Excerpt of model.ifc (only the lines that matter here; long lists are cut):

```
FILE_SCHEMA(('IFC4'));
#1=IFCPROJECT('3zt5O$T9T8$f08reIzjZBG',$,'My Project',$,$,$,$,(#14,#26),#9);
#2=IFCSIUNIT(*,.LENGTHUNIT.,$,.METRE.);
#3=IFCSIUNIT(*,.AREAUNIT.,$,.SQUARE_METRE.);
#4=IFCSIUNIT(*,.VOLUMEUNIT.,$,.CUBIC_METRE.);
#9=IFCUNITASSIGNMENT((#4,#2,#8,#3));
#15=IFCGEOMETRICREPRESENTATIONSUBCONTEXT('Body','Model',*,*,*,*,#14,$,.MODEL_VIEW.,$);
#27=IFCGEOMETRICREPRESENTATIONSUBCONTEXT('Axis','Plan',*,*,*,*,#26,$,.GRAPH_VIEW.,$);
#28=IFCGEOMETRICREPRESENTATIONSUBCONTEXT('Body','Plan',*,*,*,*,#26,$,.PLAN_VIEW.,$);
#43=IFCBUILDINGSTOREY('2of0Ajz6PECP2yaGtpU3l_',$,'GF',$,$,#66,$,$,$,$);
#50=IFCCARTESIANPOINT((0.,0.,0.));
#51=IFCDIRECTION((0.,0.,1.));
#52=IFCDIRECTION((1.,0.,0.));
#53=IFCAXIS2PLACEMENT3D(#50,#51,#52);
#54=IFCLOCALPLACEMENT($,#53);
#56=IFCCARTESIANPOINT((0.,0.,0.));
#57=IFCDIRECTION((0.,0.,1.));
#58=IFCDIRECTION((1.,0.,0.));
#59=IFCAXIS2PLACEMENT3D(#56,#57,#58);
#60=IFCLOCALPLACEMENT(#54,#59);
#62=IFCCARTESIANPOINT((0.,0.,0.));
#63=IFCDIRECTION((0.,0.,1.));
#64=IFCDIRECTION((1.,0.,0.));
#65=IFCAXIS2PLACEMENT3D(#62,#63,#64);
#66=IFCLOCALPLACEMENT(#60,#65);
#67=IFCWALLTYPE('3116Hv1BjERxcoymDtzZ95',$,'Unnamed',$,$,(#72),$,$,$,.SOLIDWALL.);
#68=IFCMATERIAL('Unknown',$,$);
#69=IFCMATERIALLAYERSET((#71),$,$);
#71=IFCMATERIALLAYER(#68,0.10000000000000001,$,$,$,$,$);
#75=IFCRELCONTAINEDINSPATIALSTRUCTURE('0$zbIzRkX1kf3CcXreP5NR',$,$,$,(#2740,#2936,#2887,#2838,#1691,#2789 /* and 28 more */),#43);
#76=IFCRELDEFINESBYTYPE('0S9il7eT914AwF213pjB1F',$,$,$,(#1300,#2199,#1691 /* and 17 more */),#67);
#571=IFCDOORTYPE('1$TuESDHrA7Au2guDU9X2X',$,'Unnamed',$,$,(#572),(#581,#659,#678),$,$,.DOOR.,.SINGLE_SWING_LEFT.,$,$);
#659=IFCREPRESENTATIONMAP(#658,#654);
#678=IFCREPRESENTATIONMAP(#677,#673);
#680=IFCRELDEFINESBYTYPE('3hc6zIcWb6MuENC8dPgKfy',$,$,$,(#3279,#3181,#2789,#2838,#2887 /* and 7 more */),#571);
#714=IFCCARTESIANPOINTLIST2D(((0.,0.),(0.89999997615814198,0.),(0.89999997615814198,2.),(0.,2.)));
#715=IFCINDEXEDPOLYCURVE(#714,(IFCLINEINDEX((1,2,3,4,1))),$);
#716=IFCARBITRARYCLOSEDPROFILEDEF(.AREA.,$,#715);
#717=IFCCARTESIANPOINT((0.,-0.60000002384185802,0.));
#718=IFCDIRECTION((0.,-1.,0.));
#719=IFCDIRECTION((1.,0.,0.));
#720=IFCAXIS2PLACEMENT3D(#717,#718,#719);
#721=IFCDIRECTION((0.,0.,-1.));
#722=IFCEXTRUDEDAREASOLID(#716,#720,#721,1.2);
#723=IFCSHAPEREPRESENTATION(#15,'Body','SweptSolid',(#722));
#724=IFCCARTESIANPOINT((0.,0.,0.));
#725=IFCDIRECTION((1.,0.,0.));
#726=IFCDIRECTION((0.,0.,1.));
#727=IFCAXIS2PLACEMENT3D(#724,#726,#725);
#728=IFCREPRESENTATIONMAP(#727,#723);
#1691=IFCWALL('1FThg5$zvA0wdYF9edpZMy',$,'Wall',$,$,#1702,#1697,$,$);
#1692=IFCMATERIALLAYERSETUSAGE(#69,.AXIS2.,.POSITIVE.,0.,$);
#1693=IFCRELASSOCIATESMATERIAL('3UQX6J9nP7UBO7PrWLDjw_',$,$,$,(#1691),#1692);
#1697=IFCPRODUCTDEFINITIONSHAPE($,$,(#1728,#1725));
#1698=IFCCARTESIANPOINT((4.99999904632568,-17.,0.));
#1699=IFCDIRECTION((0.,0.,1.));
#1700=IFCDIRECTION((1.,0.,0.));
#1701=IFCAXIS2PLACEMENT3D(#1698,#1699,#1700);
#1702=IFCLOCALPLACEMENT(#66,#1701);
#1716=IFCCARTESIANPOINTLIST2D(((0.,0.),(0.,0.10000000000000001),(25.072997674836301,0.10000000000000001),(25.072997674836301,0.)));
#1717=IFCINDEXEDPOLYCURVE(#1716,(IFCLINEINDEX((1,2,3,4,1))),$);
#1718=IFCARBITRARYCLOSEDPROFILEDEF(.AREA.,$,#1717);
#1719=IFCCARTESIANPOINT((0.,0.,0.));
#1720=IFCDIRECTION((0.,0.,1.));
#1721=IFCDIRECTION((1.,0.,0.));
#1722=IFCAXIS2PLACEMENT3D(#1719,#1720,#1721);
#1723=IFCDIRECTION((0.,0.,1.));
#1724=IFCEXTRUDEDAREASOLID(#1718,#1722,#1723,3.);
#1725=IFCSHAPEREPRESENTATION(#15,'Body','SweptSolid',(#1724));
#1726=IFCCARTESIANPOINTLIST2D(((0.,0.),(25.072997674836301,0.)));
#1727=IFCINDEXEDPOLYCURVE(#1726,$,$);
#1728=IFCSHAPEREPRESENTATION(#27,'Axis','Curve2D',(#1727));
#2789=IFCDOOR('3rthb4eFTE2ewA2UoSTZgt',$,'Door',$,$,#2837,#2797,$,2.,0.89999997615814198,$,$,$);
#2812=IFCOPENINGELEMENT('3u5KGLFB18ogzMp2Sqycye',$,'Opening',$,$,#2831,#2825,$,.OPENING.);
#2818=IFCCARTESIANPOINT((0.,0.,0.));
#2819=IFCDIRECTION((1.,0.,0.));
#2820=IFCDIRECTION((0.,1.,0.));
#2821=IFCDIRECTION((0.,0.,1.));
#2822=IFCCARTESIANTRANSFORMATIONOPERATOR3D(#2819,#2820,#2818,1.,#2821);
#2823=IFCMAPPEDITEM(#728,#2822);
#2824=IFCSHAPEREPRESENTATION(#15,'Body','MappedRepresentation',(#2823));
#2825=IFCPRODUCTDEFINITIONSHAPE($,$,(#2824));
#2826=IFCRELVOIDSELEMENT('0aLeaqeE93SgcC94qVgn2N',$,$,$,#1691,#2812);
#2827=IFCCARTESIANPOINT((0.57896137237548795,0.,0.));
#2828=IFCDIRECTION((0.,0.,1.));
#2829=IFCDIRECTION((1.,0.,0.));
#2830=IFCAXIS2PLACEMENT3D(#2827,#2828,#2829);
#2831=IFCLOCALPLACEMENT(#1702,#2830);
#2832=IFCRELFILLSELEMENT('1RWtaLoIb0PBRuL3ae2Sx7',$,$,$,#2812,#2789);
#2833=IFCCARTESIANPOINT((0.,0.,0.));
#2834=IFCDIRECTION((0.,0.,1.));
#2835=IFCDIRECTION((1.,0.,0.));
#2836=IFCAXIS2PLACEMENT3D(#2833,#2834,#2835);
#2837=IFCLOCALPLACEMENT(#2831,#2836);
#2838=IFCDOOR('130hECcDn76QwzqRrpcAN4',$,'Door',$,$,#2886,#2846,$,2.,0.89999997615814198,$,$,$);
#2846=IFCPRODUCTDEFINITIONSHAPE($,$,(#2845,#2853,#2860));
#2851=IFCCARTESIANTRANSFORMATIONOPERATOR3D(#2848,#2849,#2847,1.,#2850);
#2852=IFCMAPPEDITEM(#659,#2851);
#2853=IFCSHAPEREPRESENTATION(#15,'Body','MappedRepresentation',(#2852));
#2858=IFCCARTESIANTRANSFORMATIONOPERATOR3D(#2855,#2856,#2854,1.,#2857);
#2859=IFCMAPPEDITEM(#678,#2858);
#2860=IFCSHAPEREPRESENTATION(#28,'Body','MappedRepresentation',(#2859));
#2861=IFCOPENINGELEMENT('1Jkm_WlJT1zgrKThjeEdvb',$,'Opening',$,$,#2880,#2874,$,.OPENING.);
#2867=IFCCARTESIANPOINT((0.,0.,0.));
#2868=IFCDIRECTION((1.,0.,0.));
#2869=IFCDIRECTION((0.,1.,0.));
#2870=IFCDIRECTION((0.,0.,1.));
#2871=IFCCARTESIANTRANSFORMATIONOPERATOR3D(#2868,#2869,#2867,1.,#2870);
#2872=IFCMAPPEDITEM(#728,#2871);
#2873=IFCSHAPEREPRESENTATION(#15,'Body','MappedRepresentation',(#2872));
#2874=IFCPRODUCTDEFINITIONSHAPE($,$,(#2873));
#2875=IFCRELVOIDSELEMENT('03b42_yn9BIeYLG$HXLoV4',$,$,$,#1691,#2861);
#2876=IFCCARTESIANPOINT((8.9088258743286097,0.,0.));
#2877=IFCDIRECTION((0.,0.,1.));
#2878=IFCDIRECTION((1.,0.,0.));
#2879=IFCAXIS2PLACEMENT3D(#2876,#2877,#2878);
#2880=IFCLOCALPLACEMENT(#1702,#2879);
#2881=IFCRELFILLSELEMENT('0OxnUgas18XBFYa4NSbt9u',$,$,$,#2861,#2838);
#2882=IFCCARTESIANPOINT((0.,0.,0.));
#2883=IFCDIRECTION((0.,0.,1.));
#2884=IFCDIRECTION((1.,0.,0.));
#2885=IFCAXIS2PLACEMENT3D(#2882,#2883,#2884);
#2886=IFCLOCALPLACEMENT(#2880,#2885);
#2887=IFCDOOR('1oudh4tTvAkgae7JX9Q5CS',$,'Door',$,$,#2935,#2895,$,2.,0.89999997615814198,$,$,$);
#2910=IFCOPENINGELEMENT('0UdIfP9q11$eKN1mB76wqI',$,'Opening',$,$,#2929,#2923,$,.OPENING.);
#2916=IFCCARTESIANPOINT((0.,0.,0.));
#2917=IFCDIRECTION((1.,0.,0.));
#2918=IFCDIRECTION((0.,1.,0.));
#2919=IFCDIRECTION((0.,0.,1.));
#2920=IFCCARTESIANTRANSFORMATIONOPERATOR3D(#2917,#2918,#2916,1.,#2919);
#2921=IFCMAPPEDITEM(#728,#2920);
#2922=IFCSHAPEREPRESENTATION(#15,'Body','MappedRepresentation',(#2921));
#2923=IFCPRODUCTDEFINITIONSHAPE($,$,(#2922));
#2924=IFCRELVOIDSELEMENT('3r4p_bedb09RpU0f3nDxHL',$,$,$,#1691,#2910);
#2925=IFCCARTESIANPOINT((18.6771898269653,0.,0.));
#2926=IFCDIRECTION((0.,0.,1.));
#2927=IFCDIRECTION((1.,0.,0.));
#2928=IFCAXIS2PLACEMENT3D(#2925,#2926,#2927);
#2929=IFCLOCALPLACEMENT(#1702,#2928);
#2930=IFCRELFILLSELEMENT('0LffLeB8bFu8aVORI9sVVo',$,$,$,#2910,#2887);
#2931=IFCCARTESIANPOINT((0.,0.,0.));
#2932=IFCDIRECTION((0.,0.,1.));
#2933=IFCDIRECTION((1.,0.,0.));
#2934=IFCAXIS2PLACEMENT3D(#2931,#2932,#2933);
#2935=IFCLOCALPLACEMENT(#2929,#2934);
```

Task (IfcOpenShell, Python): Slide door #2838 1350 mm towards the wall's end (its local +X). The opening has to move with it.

```python
import ifcopenshell
import ifcopenshell.api.geometry
import ifcopenshell.util.placement
import ifcopenshell.util.unit

model = ifcopenshell.open("model.ifc")
unit_scale = ifcopenshell.util.unit.calculate_unit_scale(model)

door = model.by_id(2838)
opening = door.FillsVoids[0].RelatingOpeningElement
wall = opening.VoidsElements[0].RelatingBuildingElement

wall_matrix = ifcopenshell.util.placement.get_local_placement(wall.ObjectPlacement)
shift = wall_matrix[:3, 0] * 1.35 / unit_scale
before = ifcopenshell.util.placement.get_local_placement(door.ObjectPlacement)[:3, 3].copy()

# The door is placed relative to its opening, so it follows when the opening moves.
matrix = ifcopenshell.util.placement.get_local_placement(opening.ObjectPlacement)
matrix[:3, 3] += shift
ifcopenshell.api.geometry.edit_object_placement(
    model, product=opening, matrix=matrix, is_si=False, should_transform_children=True
)

after = ifcopenshell.util.placement.get_local_placement(door.ObjectPlacement)[:3, 3]
print("door moved by", (after - before).round(3) + 0.0)

model.write("model-out.ifc")
```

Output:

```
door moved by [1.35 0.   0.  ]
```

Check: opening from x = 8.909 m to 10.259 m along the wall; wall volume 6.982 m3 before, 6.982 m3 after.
